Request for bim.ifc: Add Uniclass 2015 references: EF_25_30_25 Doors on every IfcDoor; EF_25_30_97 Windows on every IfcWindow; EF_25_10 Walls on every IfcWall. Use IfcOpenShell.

First a look at what the model holds.

```python
import ifcopenshell

model = ifcopenshell.open("bim.ifc")
print(model.schema)
print("classifications:", [c.Name for c in model.by_type("IfcClassification")])
for ifc_class in ("IfcDoor", "IfcRoof", "IfcStair", "IfcWall", "IfcWindow"):
    print(ifc_class, len(model.by_type(ifc_class)))
```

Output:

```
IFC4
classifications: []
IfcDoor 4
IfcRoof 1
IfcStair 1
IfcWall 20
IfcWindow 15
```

```python
import ifcopenshell
import ifcopenshell.api.classification

model = ifcopenshell.open("bim.ifc")

system = ifcopenshell.api.classification.add_classification(model, classification="Uniclass 2015")

codes = {
    "IfcDoor": ("EF_25_30_25", "Doors"),
    "IfcWindow": ("EF_25_30_97", "Windows"),
    "IfcWall": ("EF_25_10", "Walls"),
}
for ifc_class, (code, name) in codes.items():
    products = model.by_type(ifc_class)
    ifcopenshell.api.classification.add_reference(
        model, products=products, classification=system, identification=code, name=name
    )
    print(code, len(products))

model.write("bim_v2.ifc")
```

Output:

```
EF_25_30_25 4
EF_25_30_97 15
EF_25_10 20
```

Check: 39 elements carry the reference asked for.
